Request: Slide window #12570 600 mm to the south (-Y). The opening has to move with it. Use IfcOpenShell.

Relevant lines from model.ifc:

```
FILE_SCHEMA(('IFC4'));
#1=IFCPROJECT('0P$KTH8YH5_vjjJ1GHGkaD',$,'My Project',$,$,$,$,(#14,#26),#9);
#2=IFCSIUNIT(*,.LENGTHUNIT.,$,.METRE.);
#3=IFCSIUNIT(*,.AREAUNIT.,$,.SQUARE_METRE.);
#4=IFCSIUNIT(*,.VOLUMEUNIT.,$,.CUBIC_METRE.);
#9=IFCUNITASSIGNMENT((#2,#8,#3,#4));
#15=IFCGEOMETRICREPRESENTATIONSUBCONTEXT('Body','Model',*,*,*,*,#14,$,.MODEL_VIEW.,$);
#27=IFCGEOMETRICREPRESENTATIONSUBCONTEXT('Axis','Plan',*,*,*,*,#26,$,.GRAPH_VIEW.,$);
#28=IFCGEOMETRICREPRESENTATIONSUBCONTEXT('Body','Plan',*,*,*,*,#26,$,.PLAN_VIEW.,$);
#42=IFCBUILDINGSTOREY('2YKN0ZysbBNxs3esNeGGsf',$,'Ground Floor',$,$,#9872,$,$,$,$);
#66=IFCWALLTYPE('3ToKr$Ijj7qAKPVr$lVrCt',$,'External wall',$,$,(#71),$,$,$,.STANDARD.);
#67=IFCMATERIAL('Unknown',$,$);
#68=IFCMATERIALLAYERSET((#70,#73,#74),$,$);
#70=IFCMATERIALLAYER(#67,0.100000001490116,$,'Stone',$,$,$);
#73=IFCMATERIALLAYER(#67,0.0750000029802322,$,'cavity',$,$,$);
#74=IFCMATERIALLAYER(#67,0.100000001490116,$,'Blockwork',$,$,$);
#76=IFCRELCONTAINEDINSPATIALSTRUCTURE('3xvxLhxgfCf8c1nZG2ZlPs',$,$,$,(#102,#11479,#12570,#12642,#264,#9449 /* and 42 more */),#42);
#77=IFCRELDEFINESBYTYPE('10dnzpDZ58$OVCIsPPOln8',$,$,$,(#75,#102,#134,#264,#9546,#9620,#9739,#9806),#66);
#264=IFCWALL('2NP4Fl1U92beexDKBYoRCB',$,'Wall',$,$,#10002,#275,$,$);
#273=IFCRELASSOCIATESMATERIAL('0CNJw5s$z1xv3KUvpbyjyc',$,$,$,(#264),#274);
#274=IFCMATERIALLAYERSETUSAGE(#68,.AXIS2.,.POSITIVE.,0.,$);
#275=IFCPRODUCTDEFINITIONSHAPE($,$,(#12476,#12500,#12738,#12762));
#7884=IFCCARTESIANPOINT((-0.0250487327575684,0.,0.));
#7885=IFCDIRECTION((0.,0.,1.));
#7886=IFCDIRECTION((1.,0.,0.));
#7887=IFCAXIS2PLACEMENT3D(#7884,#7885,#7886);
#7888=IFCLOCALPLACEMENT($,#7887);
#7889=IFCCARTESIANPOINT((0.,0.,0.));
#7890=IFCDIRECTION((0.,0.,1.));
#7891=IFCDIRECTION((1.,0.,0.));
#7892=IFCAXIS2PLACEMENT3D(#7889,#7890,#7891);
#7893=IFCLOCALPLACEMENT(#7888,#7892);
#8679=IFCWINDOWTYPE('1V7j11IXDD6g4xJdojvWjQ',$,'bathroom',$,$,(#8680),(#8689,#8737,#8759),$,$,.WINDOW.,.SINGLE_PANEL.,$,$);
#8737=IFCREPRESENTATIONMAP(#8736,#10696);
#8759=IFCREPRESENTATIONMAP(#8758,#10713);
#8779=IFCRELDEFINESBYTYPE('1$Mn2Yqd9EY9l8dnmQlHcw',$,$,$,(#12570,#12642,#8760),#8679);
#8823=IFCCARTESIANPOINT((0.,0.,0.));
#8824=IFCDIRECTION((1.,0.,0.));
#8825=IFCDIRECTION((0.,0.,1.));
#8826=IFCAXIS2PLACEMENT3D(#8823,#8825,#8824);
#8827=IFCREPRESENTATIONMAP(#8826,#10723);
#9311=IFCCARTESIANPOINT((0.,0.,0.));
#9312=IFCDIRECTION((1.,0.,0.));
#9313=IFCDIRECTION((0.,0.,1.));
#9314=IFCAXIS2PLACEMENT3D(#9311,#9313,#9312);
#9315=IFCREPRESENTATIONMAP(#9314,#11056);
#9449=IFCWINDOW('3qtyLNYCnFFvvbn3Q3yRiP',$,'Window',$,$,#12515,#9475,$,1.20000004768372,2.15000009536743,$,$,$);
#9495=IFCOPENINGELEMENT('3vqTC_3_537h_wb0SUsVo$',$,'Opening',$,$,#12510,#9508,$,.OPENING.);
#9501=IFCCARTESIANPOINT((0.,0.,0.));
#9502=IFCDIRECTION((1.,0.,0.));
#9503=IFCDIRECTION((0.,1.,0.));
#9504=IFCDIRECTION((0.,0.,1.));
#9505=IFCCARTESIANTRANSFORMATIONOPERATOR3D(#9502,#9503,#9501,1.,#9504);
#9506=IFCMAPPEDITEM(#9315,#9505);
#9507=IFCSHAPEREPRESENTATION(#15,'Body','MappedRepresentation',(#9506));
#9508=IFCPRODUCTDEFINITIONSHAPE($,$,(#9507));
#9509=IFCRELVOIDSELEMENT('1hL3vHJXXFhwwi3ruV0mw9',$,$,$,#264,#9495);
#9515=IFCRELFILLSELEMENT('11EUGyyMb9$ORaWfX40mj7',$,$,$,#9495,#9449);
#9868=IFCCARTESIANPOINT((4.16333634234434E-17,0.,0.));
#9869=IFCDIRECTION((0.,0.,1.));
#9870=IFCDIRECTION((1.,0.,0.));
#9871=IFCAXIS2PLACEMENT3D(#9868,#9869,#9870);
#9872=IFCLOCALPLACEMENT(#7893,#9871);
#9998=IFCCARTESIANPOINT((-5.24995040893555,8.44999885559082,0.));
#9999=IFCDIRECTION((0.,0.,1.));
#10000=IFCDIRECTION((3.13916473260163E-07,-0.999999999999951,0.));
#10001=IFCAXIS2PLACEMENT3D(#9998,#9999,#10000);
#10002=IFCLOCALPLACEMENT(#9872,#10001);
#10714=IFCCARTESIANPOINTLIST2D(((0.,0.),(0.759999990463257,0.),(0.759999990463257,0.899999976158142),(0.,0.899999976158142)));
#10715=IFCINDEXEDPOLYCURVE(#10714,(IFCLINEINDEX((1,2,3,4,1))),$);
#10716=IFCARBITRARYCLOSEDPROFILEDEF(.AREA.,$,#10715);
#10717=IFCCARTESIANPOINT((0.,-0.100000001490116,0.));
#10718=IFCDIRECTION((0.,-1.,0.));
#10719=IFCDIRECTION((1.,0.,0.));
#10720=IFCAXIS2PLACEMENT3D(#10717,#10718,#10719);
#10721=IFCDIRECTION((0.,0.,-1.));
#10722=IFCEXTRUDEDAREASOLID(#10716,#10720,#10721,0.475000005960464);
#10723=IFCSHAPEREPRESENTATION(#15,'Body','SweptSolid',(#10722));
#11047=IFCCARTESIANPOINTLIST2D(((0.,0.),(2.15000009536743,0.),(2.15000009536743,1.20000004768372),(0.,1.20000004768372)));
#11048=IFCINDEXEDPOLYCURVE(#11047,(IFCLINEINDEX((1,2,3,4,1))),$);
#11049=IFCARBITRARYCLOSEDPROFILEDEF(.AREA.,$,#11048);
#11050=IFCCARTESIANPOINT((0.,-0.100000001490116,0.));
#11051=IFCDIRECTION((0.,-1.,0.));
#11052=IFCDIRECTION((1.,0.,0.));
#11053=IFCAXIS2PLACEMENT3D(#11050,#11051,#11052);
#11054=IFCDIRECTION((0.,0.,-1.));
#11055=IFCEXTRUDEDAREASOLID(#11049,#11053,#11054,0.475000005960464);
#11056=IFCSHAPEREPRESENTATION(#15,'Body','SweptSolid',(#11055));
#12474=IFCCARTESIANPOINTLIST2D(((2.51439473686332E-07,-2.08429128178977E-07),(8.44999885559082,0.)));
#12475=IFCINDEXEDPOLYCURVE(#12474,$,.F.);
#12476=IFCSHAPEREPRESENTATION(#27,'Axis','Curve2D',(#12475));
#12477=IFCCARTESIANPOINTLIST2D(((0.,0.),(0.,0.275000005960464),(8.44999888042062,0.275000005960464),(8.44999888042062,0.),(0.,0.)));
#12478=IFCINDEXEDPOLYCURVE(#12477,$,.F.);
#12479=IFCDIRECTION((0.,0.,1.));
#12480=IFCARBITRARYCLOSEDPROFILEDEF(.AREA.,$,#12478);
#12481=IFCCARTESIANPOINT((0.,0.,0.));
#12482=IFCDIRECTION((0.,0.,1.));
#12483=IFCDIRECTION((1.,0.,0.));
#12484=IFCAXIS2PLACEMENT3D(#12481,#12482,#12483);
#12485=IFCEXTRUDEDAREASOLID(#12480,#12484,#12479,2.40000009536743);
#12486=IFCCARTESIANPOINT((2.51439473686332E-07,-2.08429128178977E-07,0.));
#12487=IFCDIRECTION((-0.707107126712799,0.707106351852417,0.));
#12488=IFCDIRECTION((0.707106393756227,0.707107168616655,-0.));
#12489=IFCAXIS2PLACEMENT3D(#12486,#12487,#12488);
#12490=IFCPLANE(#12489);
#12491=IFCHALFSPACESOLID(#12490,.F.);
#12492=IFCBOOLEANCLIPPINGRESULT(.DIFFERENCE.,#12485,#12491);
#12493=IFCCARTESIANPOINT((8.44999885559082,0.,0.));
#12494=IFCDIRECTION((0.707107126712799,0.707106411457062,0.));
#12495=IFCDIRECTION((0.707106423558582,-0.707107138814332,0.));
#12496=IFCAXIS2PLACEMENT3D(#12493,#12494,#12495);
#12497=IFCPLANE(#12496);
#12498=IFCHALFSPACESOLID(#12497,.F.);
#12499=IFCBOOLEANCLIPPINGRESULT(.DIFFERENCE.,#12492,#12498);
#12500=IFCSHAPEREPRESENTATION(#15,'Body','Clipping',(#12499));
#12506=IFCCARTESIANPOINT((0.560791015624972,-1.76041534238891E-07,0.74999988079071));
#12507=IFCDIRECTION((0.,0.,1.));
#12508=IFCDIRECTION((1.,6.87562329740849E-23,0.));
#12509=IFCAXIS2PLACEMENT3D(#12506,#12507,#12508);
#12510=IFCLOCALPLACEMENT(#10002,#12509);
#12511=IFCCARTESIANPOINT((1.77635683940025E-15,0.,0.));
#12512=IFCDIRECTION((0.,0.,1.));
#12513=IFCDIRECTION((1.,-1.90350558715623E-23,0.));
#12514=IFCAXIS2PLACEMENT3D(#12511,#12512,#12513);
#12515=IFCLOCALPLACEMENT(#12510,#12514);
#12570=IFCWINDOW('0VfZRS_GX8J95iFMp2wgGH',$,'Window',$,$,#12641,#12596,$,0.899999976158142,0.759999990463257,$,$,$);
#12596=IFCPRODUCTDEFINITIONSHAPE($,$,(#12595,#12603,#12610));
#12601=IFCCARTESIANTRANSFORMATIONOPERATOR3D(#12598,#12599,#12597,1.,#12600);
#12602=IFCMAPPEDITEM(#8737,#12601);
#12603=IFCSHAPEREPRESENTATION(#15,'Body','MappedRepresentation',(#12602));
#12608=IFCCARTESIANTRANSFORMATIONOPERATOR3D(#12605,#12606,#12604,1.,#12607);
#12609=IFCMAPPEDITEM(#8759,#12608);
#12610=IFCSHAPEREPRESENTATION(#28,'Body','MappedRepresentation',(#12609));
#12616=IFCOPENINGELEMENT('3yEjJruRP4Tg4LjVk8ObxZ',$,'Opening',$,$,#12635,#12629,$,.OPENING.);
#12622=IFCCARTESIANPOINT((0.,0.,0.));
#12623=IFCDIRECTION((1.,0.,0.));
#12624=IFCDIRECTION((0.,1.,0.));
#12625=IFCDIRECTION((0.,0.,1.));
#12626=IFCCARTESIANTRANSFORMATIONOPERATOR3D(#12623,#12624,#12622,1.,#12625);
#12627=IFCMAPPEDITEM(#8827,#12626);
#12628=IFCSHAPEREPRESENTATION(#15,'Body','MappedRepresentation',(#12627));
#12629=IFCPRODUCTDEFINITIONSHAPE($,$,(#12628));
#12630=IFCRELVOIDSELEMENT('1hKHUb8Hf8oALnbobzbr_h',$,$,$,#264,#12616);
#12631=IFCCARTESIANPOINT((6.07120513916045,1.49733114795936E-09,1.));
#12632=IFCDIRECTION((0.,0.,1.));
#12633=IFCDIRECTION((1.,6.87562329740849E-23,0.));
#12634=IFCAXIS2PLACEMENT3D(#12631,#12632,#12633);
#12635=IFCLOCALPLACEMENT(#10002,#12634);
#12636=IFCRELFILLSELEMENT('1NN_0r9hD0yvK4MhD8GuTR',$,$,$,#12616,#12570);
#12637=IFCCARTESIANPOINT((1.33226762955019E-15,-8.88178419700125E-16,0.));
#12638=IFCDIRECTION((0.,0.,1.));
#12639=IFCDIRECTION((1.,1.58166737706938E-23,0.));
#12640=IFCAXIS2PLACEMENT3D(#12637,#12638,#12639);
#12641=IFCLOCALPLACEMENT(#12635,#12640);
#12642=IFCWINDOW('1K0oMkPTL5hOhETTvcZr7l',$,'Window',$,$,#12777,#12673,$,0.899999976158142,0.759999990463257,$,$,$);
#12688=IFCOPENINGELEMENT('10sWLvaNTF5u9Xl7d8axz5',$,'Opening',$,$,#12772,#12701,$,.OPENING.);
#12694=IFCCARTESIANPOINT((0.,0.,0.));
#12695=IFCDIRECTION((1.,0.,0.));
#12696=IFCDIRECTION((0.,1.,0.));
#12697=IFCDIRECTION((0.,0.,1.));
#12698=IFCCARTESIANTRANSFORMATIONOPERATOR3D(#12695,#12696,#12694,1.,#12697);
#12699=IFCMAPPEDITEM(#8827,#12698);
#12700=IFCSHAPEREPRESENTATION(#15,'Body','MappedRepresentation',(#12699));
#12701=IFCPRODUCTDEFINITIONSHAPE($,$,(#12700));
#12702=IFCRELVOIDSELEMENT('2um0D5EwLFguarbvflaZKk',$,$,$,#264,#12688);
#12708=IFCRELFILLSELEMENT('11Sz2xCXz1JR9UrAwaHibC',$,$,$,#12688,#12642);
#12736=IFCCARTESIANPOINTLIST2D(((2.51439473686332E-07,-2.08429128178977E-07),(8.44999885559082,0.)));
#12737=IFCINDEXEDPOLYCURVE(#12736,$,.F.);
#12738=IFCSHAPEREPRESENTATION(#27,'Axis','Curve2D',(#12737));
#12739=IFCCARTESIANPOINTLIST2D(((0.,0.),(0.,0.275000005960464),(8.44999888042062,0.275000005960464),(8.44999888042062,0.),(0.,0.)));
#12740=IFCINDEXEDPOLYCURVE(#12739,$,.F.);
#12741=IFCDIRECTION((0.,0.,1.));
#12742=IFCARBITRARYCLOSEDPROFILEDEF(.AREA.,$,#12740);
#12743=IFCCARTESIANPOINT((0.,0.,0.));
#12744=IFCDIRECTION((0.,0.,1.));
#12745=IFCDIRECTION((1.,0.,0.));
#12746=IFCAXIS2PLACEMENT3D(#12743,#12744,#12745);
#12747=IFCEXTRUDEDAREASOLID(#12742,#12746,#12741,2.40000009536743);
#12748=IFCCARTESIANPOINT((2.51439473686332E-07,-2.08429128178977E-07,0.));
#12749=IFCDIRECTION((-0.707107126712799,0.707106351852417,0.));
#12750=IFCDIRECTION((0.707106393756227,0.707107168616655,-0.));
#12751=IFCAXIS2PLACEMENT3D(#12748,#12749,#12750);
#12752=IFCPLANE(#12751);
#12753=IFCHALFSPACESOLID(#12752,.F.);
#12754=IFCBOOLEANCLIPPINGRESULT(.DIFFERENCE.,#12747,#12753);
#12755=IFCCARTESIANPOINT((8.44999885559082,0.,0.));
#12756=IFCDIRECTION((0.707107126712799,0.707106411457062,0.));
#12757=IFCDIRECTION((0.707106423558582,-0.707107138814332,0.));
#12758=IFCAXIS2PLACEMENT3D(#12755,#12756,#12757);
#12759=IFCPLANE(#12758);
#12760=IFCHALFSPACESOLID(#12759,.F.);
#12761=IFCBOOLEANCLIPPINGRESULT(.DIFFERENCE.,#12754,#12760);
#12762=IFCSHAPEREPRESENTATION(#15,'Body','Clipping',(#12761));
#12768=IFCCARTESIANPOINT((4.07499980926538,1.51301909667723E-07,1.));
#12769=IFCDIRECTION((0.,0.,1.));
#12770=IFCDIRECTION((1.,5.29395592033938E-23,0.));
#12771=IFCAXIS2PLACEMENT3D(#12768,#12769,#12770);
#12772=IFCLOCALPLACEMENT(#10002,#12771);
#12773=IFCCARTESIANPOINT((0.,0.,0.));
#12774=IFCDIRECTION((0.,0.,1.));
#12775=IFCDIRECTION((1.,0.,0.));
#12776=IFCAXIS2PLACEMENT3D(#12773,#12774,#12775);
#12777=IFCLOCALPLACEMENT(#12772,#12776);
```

```python
import ifcopenshell
import ifcopenshell.api.geometry
import ifcopenshell.util.placement
import ifcopenshell.util.unit

model = ifcopenshell.open("model.ifc")
unit_scale = ifcopenshell.util.unit.calculate_unit_scale(model)

window = model.by_guid("0VfZRS_GX8J95iFMp2wgGH")
opening = window.FillsVoids[0].RelatingOpeningElement
wall = opening.VoidsElements[0].RelatingBuildingElement

wall_matrix = ifcopenshell.util.placement.get_local_placement(wall.ObjectPlacement)
shift = wall_matrix[:3, 0] * 0.6 / unit_scale
before = ifcopenshell.util.placement.get_local_placement(window.ObjectPlacement)[:3, 3].copy()

# The window is placed relative to its opening, so it follows when the opening moves.
matrix = ifcopenshell.util.placement.get_local_placement(opening.ObjectPlacement)
matrix[:3, 3] += shift
ifcopenshell.api.geometry.edit_object_placement(
    model, product=opening, matrix=matrix, is_si=False, should_transform_children=True
)

after = ifcopenshell.util.placement.get_local_placement(window.ObjectPlacement)[:3, 3]
print("window moved by", (after - before).round(3) + 0.0)

model.write("model_rev.ifc")
```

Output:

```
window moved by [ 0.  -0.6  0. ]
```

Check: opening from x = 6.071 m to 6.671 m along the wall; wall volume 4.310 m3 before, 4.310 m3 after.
